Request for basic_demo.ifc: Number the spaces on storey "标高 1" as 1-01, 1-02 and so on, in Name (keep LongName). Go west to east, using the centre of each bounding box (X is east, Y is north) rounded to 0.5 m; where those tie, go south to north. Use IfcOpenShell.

First a look at what the model holds.

```python
import ifcopenshell
import ifcopenshell.util.element
import ifcopenshell.util.placement

model = ifcopenshell.open("basic_demo.ifc")
print(model.schema)
storey = next(s for s in model.by_type("IfcBuildingStorey") if s.Name == "标高 1")
spaces = [e for e in ifcopenshell.util.element.get_decomposition(storey) if e.is_a("IfcSpace")]
for e in sorted(spaces, key=lambda e: e.id()):
    origin = ifcopenshell.util.placement.get_local_placement(e.ObjectPlacement)[:3, 3]
    print(e.id(), e.Name, e.LongName, origin.round(2) + 0.0, sep=" | ")
```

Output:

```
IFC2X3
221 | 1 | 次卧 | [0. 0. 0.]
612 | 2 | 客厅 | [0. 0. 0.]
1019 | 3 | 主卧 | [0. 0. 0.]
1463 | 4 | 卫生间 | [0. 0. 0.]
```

```python
import ifcopenshell
import ifcopenshell.geom
import ifcopenshell.util.element
import ifcopenshell.util.shape

model = ifcopenshell.open("basic_demo.ifc")
settings = ifcopenshell.geom.settings()
settings.set("use-world-coords", True)


def centre(element):
    shape = ifcopenshell.geom.create_shape(settings, element)
    return ifcopenshell.util.shape.get_bbox_centroid(shape.geometry)


storey = next(s for s in model.by_type("IfcBuildingStorey") if s.Name == "标高 1")
spaces = [e for e in ifcopenshell.util.element.get_decomposition(storey) if e.is_a("IfcSpace")]

# Insertion points can sit at a corner or the storey origin, so sort by the geometry (in metres).
centres = {e: centre(e) for e in spaces}
spaces.sort(key=lambda e: (round(centres[e][0] / 0.5), centres[e][1]))

for i, e in enumerate(spaces, start=1):
    number = f"1-{i:02d}"
    e.Name = number
    print(e.id(), number)

model.write("basic_demo_rev.ifc")
```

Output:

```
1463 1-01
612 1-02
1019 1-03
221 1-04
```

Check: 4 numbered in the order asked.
